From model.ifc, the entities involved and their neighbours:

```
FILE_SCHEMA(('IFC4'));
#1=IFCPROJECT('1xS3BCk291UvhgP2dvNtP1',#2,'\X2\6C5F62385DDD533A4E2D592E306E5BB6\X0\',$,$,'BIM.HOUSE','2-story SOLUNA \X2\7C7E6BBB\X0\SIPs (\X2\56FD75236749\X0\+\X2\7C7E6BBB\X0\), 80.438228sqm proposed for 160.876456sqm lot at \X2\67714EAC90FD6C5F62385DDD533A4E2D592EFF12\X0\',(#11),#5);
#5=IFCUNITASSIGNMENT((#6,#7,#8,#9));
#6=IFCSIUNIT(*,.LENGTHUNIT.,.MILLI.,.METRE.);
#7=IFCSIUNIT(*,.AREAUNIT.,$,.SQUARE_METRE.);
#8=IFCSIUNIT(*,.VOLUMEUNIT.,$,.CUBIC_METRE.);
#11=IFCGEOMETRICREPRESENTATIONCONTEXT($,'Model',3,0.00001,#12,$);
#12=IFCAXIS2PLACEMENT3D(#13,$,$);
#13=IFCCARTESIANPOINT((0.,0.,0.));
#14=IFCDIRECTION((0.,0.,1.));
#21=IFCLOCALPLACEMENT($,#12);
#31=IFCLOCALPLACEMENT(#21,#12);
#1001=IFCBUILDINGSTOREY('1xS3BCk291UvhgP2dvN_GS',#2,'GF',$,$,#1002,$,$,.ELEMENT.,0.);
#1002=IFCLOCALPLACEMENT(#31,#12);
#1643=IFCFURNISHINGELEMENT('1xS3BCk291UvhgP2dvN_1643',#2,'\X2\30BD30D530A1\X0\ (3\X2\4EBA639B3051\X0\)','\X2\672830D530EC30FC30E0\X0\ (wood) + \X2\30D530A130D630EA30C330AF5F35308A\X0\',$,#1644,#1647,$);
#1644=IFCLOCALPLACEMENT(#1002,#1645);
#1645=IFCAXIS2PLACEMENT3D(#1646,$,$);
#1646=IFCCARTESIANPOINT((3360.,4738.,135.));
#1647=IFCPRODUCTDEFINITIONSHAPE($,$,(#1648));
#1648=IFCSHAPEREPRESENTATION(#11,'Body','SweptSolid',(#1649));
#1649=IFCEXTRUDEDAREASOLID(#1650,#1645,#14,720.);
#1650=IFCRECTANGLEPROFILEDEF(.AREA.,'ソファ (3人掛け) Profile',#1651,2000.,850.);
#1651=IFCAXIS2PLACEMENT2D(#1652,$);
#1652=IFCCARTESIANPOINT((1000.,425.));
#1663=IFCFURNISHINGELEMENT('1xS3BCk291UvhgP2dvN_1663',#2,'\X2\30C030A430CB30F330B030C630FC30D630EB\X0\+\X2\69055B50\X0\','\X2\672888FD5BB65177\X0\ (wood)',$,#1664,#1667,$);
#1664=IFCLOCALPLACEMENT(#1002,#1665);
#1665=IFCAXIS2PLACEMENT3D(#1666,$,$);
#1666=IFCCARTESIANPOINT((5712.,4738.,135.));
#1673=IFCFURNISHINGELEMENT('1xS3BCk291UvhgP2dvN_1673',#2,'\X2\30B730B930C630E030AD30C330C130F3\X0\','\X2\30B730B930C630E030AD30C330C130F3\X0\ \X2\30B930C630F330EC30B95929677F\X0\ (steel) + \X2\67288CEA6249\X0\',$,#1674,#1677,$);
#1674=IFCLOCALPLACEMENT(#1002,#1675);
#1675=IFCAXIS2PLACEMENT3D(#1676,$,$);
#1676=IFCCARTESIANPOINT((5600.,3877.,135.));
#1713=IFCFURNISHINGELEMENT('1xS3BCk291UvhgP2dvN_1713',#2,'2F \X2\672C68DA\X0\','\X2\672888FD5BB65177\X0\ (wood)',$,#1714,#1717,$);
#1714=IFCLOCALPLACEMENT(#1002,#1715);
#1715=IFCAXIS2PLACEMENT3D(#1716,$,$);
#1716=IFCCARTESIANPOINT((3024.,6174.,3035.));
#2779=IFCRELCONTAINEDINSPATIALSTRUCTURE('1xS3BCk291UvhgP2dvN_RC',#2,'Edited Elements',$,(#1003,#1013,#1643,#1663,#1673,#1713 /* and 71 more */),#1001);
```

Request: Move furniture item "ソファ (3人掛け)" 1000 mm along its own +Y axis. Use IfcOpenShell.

```python
import ifcopenshell
import ifcopenshell.api.geometry
import ifcopenshell.util.placement
import ifcopenshell.util.unit

model = ifcopenshell.open("model.ifc")
unit_scale = ifcopenshell.util.unit.calculate_unit_scale(model)

item = model.by_guid("1xS3BCk291UvhgP2dvN_1643")
matrix = ifcopenshell.util.placement.get_local_placement(item.ObjectPlacement)
matrix[:3, 3] += matrix[:3, 1] * 1 / unit_scale
ifcopenshell.api.geometry.edit_object_placement(model, product=item, matrix=matrix, is_si=False)

print(ifcopenshell.util.placement.get_local_placement(item.ObjectPlacement).round(3) + 0.0)

model.write("model-out.ifc")
```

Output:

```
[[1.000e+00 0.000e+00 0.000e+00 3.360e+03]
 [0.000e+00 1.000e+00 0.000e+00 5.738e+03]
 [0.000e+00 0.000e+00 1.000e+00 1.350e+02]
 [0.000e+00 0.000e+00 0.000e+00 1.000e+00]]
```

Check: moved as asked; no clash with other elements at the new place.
